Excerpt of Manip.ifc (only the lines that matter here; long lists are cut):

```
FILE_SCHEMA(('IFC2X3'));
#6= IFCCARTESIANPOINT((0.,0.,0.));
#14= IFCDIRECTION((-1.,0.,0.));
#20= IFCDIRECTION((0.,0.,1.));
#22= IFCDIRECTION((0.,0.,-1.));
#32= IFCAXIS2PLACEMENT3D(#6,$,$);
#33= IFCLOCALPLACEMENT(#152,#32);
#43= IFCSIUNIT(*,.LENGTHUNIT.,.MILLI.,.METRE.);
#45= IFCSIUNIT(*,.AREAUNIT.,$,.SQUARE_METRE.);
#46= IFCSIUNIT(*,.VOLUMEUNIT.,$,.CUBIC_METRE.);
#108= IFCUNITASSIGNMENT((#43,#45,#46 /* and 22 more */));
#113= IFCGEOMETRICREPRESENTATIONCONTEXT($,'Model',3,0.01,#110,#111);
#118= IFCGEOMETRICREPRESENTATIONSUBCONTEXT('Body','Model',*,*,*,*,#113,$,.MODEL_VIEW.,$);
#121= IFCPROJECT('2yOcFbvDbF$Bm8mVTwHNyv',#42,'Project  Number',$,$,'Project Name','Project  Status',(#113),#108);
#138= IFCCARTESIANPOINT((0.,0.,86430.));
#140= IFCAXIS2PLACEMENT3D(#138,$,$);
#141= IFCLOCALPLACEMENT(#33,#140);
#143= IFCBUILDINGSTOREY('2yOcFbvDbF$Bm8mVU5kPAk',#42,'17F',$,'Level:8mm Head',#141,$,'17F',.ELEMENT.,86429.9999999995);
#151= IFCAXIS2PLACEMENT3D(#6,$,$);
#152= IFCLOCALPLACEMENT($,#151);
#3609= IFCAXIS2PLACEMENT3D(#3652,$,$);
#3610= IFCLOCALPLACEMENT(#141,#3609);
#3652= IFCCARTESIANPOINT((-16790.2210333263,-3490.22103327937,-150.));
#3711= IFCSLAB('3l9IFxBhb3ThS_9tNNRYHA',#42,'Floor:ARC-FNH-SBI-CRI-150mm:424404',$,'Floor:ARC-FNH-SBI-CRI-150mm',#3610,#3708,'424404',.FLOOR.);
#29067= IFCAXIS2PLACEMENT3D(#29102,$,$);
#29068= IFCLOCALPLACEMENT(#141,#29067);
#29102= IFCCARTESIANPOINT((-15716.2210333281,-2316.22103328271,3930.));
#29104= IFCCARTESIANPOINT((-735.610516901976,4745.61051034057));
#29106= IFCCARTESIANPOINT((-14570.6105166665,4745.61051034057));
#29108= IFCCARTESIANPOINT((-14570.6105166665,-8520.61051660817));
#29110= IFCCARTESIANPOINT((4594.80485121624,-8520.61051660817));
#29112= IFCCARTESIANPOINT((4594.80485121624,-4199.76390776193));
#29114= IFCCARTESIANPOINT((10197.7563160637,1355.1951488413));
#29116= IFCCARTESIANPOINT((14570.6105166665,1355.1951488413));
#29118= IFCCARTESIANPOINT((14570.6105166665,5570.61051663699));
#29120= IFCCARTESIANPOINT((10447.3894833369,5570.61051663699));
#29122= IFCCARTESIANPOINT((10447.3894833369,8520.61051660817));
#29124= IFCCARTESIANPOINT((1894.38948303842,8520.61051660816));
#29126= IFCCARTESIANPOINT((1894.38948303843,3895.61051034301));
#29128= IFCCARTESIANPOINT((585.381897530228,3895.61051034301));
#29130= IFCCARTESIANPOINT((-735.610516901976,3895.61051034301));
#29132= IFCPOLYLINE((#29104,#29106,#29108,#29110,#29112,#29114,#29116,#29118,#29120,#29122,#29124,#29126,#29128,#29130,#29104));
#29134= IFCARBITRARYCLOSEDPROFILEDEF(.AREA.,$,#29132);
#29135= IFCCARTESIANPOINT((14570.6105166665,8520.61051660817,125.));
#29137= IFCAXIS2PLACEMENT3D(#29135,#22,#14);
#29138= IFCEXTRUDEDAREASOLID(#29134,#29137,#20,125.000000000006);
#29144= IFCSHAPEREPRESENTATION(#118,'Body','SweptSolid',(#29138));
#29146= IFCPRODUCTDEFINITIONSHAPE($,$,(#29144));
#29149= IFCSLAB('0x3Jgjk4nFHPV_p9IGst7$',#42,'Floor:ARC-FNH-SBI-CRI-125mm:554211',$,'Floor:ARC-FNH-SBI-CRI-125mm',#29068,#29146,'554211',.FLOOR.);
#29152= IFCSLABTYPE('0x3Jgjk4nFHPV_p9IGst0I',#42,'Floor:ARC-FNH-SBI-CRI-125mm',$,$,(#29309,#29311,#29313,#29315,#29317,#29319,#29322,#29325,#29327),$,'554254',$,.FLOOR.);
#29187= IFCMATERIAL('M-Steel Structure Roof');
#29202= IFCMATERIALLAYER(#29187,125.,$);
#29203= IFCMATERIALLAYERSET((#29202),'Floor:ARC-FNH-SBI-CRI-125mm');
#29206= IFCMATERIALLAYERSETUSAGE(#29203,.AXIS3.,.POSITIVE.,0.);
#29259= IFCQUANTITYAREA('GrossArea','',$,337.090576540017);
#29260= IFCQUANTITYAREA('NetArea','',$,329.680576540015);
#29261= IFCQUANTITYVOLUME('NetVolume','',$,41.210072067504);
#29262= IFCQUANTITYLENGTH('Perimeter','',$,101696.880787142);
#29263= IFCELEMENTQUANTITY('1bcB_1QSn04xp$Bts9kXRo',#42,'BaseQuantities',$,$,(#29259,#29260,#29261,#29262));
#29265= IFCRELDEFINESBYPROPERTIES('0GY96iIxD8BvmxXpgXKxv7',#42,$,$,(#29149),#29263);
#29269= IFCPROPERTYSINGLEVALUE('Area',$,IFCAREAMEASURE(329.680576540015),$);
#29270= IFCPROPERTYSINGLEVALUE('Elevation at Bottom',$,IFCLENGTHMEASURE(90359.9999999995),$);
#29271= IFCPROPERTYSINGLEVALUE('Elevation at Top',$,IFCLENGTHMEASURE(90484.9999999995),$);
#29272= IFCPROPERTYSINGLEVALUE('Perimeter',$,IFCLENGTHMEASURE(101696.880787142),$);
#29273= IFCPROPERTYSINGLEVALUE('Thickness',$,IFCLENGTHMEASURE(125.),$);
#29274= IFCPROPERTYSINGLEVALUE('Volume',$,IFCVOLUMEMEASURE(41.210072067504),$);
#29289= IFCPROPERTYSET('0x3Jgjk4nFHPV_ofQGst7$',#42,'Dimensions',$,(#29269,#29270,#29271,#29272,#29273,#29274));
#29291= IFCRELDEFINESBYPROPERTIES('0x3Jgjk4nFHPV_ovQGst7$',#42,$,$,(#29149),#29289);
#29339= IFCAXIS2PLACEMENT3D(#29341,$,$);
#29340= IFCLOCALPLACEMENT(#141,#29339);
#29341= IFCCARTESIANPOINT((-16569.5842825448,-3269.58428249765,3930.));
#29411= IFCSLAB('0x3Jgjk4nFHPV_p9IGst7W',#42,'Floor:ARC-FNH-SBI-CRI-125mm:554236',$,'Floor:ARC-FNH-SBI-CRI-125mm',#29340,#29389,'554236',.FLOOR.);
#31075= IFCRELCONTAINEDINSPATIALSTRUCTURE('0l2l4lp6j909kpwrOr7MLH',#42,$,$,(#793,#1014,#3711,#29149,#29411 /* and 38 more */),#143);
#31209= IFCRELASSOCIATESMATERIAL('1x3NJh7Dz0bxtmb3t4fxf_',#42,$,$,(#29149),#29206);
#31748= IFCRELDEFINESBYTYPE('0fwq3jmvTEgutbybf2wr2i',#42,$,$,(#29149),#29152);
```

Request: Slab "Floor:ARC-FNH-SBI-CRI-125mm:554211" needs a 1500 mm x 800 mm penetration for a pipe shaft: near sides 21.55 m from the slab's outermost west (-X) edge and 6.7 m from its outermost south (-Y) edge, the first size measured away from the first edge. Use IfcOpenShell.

```python
import numpy as np
import ifcopenshell
import ifcopenshell.api.feature
import ifcopenshell.api.geometry
import ifcopenshell.api.pset
import ifcopenshell.api.root
import ifcopenshell.geom
import ifcopenshell.util.element
import ifcopenshell.util.placement
import ifcopenshell.util.representation
import ifcopenshell.util.shape
import ifcopenshell.util.unit

model = ifcopenshell.open("Manip.ifc")
unit_scale = ifcopenshell.util.unit.calculate_unit_scale(model)
area_scale = ifcopenshell.util.unit.calculate_unit_scale(model, "AREAUNIT")
volume_scale = ifcopenshell.util.unit.calculate_unit_scale(model, "VOLUMEUNIT")
settings = ifcopenshell.geom.settings()


def volume(element):
    """Net volume in cubic metres, openings subtracted."""
    shape = ifcopenshell.geom.create_shape(settings, element)
    return ifcopenshell.util.shape.get_volume(shape.geometry)


slab = model.by_guid("0x3Jgjk4nFHPV_p9IGst7$")
before = volume(slab)

# Extent in the slab's own axes, in metres. The edges named are its -X and -Y sides.
slab_shape = ifcopenshell.geom.create_shape(settings, slab)
vertices = ifcopenshell.util.shape.get_vertices(slab_shape.geometry)
x_min, y_min, bottom = vertices.min(axis=0)
top = vertices[:, 2].max()

opening = ifcopenshell.api.root.create_entity(model, ifc_class="IfcOpeningElement", name="Pipe shaft opening")
context = ifcopenshell.util.representation.get_context(model, "Model", "Body", "MODEL_VIEW")
width, depth = 1.5, 0.8
outline = [(0.0, 0.0), (width, 0.0), (width, depth), (0.0, depth), (0.0, 0.0)]
# Overshoot both faces by 50 mm so the cut is clean.
shape = ifcopenshell.api.geometry.add_slab_representation(
    model, context=context, depth=top - bottom + 0.1, polyline=outline
)
ifcopenshell.api.geometry.assign_representation(model, product=opening, representation=shape)

matrix = ifcopenshell.util.placement.get_local_placement(slab.ObjectPlacement)
matrix[:, 3] = matrix @ np.append(np.array([x_min + 21.55, y_min + 6.7, bottom - 0.05]) / unit_scale, 1.0)
ifcopenshell.api.geometry.edit_object_placement(model, product=opening, matrix=matrix, is_si=False)
ifcopenshell.api.feature.add_feature(model, feature=opening, element=slab)

after = volume(slab)

# Update the slab's stored quantities.
qto = model.by_id(ifcopenshell.util.element.get_pset(slab, "BaseQuantities", should_inherit=False)["id"])
ifcopenshell.api.pset.edit_qto(model, qto=qto, properties={
    "NetArea": after / (top - bottom) / area_scale,
    "NetVolume": after / volume_scale,
})
pset = model.by_id(ifcopenshell.util.element.get_pset(slab, "Dimensions", should_inherit=False)["id"])
ifcopenshell.api.pset.edit_pset(model, pset=pset, properties={
    "Area": model.create_entity("IfcAreaMeasure", after / (top - bottom) / area_scale),
    "Volume": model.create_entity("IfcVolumeMeasure", after / volume_scale),
})

print(f"slab volume {before:.3f} -> {after:.3f} m3")

model.write("Manip-out.ifc")
```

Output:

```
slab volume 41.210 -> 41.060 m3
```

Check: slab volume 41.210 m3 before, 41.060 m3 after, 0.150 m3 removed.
